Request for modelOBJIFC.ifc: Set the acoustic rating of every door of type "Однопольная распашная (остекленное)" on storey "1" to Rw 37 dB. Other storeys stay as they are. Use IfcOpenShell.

First a look at what the model holds.

```python
import ifcopenshell
import ifcopenshell.util.element

model = ifcopenshell.open("modelOBJIFC.ifc")
print(model.schema)
storey = next(s for s in model.by_type("IfcBuildingStorey") if s.Name == "1")
doors = [e for e in ifcopenshell.util.element.get_decomposition(storey) if e.is_a("IfcDoor")]
seen = {}
for e in doors:
    element_type = ifcopenshell.util.element.get_type(e)
    key = (element_type.Name if element_type != e and element_type else None, ifcopenshell.util.element.get_pset(e, "Pset_DoorCommon", "AcousticRating"))
    seen[key] = seen.get(key, 0) + 1
for (name, value), count in sorted(seen.items(), key=str):
    print(count, "x", name, "|", value)
```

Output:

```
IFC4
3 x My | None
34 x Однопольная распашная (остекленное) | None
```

```python
import ifcopenshell
import ifcopenshell.api.pset
import ifcopenshell.util.element

model = ifcopenshell.open("modelOBJIFC.ifc")

storey = next(s for s in model.by_type("IfcBuildingStorey") if s.Name == "1")
doors = [e for e in ifcopenshell.util.element.get_decomposition(storey) if e.is_a("IfcDoor")]

count = 0
for e in doors:
    element_type = ifcopenshell.util.element.get_type(e)
    if element_type in (None, e) or element_type.Name != "Однопольная распашная (остекленное)":
        continue
    # add_pset returns the element's existing set when there is one.
    pset = ifcopenshell.api.pset.add_pset(model, product=e, name="Pset_DoorCommon")
    ifcopenshell.api.pset.edit_pset(model, pset=pset, properties={"AcousticRating": "Rw 37 dB"})
    count += 1

print(count, "doors updated")

model.write("modelOBJIFC_edited.ifc")
```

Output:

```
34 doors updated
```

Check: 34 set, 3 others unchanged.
